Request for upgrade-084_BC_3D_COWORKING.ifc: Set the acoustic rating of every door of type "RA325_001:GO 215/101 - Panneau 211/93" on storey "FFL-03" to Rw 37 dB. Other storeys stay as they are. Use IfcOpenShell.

First a look at what the model holds.

```python
import ifcopenshell
import ifcopenshell.util.element

model = ifcopenshell.open("upgrade-084_BC_3D_COWORKING.ifc")
print(model.schema)
storey = next(s for s in model.by_type("IfcBuildingStorey") if s.Name == "FFL-03")
doors = [e for e in ifcopenshell.util.element.get_decomposition(storey) if e.is_a("IfcDoor")]
seen = {}
for e in doors:
    element_type = ifcopenshell.util.element.get_type(e)
    key = (element_type.Name if element_type != e and element_type else None, ifcopenshell.util.element.get_pset(e, "Pset_DoorCommon", "AcousticRating"))
    seen[key] = seen.get(key, 0) + 1
for (name, value), count in sorted(seen.items(), key=str):
    print(count, "x", name, "|", value)
```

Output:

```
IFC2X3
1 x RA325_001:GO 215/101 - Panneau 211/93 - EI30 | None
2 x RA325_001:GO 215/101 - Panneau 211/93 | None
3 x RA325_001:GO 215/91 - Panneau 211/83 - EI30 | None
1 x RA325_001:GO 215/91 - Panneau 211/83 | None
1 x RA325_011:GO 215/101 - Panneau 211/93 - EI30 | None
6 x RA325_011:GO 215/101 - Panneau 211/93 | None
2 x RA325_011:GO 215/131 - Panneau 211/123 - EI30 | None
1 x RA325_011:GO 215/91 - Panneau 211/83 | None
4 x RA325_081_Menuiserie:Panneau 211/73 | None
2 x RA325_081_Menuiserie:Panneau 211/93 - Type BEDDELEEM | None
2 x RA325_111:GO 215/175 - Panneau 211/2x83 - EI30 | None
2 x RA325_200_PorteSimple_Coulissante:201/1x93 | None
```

```python
import ifcopenshell
import ifcopenshell.api.pset
import ifcopenshell.util.element

model = ifcopenshell.open("upgrade-084_BC_3D_COWORKING.ifc")

storey = next(s for s in model.by_type("IfcBuildingStorey") if s.Name == "FFL-03")
doors = [e for e in ifcopenshell.util.element.get_decomposition(storey) if e.is_a("IfcDoor")]

count = 0
for e in doors:
    element_type = ifcopenshell.util.element.get_type(e)
    if element_type in (None, e) or element_type.Name != "RA325_001:GO 215/101 - Panneau 211/93":
        continue
    # add_pset returns the element's existing set when there is one.
    pset = ifcopenshell.api.pset.add_pset(model, product=e, name="Pset_DoorCommon")
    ifcopenshell.api.pset.edit_pset(model, pset=pset, properties={"AcousticRating": "Rw 37 dB"})
    count += 1

print(count, "doors updated")

model.write("upgrade-084_BC_3D_COWORKING-out.ifc")
```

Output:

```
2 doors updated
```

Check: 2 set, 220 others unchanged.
